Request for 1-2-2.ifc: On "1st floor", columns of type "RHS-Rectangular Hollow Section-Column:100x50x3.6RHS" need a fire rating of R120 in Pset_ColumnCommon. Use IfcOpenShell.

First a look at what the model holds.

```python
import ifcopenshell
import ifcopenshell.util.element

model = ifcopenshell.open("1-2-2.ifc")
print(model.schema)
storey = next(s for s in model.by_type("IfcBuildingStorey") if s.Name == "1st floor")
columns = [e for e in ifcopenshell.util.element.get_decomposition(storey) if e.is_a("IfcColumn")]
seen = {}
for e in columns:
    element_type = ifcopenshell.util.element.get_type(e)
    key = (element_type.Name if element_type != e and element_type else None, ifcopenshell.util.element.get_pset(e, "Pset_ColumnCommon", "FireRating"))
    seen[key] = seen.get(key, 0) + 1
for (name, value), count in sorted(seen.items(), key=str):
    print(count, "x", name, "|", value)
```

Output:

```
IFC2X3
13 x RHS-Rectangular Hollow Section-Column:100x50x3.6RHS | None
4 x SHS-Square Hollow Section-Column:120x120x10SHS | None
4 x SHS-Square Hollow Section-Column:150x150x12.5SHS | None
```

```python
import ifcopenshell
import ifcopenshell.api.pset
import ifcopenshell.util.element

model = ifcopenshell.open("1-2-2.ifc")

storey = next(s for s in model.by_type("IfcBuildingStorey") if s.Name == "1st floor")
columns = [e for e in ifcopenshell.util.element.get_decomposition(storey) if e.is_a("IfcColumn")]

count = 0
for e in columns:
    element_type = ifcopenshell.util.element.get_type(e)
    if element_type in (None, e) or element_type.Name != "RHS-Rectangular Hollow Section-Column:100x50x3.6RHS":
        continue
    # add_pset returns the element's existing set when there is one.
    pset = ifcopenshell.api.pset.add_pset(model, product=e, name="Pset_ColumnCommon")
    ifcopenshell.api.pset.edit_pset(model, pset=pset, properties={"FireRating": "R120"})
    count += 1

print(count, "columns updated")

model.write("1-2-2-out.ifc")
```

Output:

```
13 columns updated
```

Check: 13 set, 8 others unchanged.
